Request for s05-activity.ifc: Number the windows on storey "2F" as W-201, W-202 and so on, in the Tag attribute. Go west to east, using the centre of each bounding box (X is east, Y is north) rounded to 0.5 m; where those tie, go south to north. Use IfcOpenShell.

First a look at what the model holds.

```python
import ifcopenshell
import ifcopenshell.util.element
import ifcopenshell.util.placement

model = ifcopenshell.open("s05-activity.ifc")
print(model.schema)
storey = next(s for s in model.by_type("IfcBuildingStorey") if s.Name == "2F")
windows = [e for e in ifcopenshell.util.element.get_decomposition(storey) if e.is_a("IfcWindow")]
for e in sorted(windows, key=lambda e: e.id()):
    origin = ifcopenshell.util.placement.get_local_placement(e.ObjectPlacement)[:3, 3]
    print(e.id(), e.Tag, e.Name, origin.round(2) + 0.0, sep=" | ")
```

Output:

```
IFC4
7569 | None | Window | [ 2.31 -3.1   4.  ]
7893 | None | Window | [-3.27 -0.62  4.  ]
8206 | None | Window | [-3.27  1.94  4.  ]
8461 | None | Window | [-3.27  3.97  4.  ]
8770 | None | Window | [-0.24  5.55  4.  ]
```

```python
import ifcopenshell
import ifcopenshell.geom
import ifcopenshell.util.element
import ifcopenshell.util.shape

model = ifcopenshell.open("s05-activity.ifc")
settings = ifcopenshell.geom.settings()
settings.set("use-world-coords", True)


def centre(element):
    shape = ifcopenshell.geom.create_shape(settings, element)
    return ifcopenshell.util.shape.get_bbox_centroid(shape.geometry)


storey = next(s for s in model.by_type("IfcBuildingStorey") if s.Name == "2F")
windows = [e for e in ifcopenshell.util.element.get_decomposition(storey) if e.is_a("IfcWindow")]

# Insertion points can sit at a corner or the storey origin, so sort by the geometry (in metres).
centres = {e: centre(e) for e in windows}
windows.sort(key=lambda e: (round(centres[e][0] / 0.5), centres[e][1]))

for i, e in enumerate(windows, start=1):
    number = f"W-2{i:02d}"
    e.Tag = number
    print(e.id(), number)

model.write("s05-activity_updated.ifc")
```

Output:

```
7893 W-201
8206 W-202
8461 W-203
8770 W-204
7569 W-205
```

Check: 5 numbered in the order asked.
